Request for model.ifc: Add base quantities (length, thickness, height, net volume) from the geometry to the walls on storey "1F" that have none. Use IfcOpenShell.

First a look at what the model holds.

```python
import ifcopenshell
import ifcopenshell.util.element
import ifcopenshell.util.unit

model = ifcopenshell.open("model.ifc")
print(model.schema)
for unit_type in ("LENGTHUNIT", "AREAUNIT", "VOLUMEUNIT"):
    print(unit_type, ifcopenshell.util.unit.calculate_unit_scale(model, unit_type))
storey = next(s for s in model.by_type("IfcBuildingStorey") if s.Name == "1F")
walls = [e for e in ifcopenshell.util.element.get_decomposition(storey) if e.is_a("IfcWall")]
for e in sorted(walls, key=lambda e: e.id()):
    print(e.id(), e.is_a(), e.Name, list(ifcopenshell.util.element.get_psets(e, qtos_only=True)), sep=" | ")
```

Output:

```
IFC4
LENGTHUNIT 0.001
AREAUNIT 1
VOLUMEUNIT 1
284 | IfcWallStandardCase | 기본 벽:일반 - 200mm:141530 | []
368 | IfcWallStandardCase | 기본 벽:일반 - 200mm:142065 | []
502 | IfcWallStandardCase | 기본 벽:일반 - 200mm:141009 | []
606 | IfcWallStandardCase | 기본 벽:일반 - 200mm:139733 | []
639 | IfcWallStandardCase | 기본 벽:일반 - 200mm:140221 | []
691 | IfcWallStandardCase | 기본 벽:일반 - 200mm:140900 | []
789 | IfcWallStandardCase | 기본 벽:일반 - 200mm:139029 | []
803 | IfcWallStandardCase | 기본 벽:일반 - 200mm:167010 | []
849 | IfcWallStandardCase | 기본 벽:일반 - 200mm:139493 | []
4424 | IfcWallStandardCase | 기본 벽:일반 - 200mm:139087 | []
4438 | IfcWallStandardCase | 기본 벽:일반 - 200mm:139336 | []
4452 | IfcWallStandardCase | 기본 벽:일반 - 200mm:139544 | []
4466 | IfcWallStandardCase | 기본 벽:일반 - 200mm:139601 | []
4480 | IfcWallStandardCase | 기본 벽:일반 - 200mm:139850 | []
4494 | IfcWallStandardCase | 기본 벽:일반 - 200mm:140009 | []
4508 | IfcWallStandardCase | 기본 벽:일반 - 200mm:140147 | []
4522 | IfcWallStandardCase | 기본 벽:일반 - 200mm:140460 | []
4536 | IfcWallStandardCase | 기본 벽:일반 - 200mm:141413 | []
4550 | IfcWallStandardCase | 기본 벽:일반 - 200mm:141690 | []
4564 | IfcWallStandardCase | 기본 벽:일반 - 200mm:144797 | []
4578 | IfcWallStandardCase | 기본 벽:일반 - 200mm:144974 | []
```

```python
import ifcopenshell
import ifcopenshell.api.pset
import ifcopenshell.geom
import ifcopenshell.util.element
import ifcopenshell.util.shape
import ifcopenshell.util.unit

model = ifcopenshell.open("model.ifc")
unit_scale = ifcopenshell.util.unit.calculate_unit_scale(model)
volume_scale = ifcopenshell.util.unit.calculate_unit_scale(model, "VOLUMEUNIT")
settings = ifcopenshell.geom.settings()

storey = next(s for s in model.by_type("IfcBuildingStorey") if s.Name == "1F")
walls = [e for e in ifcopenshell.util.element.get_decomposition(storey) if e.is_a("IfcWall")]

for e in sorted(walls, key=lambda e: e.id()):
    if ifcopenshell.util.element.get_psets(e, qtos_only=True, should_inherit=False):
        continue
    # Geometry comes back in metres, in the element's own axes.
    shape = ifcopenshell.geom.create_shape(settings, e)
    values = {
        "Length": ifcopenshell.util.shape.get_x(shape.geometry) / unit_scale,
        "Width": ifcopenshell.util.shape.get_y(shape.geometry) / unit_scale,
        "Height": ifcopenshell.util.shape.get_z(shape.geometry) / unit_scale,
        "NetVolume": ifcopenshell.util.shape.get_volume(shape.geometry) / volume_scale,
    }
    qto = ifcopenshell.api.pset.add_qto(model, product=e, name="Qto_WallBaseQuantities")
    ifcopenshell.api.pset.edit_qto(model, qto=qto, properties=values)
    print(e.id(), {k: round(v, 3) for k, v in values.items()})

model.write("model_updated.ifc")
```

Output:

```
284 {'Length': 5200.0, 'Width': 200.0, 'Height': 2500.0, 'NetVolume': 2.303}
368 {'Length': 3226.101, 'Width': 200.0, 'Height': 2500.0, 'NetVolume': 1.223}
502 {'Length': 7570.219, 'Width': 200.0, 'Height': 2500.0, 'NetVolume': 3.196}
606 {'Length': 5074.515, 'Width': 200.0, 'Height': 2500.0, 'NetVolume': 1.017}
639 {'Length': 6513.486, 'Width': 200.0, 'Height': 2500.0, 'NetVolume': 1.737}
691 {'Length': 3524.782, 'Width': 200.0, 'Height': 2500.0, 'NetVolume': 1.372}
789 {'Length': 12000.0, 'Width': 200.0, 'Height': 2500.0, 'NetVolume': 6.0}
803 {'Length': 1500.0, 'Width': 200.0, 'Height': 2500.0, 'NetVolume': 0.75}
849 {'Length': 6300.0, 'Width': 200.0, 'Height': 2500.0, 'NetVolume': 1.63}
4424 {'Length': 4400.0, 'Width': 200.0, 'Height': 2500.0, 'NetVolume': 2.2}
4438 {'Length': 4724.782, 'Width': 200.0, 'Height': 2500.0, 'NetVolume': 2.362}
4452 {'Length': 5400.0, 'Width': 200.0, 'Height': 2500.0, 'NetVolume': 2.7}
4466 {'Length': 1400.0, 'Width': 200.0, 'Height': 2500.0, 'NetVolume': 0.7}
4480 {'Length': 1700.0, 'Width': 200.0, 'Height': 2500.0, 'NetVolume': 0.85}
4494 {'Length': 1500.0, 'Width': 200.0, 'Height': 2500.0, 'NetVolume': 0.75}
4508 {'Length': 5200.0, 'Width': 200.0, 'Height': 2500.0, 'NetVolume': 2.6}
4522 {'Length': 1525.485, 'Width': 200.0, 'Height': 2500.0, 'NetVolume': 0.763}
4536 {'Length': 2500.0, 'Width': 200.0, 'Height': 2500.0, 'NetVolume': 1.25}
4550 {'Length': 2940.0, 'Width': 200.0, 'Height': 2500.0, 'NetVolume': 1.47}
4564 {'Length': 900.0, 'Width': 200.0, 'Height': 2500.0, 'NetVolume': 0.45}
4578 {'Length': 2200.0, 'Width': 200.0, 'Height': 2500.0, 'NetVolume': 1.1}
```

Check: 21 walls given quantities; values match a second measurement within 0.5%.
